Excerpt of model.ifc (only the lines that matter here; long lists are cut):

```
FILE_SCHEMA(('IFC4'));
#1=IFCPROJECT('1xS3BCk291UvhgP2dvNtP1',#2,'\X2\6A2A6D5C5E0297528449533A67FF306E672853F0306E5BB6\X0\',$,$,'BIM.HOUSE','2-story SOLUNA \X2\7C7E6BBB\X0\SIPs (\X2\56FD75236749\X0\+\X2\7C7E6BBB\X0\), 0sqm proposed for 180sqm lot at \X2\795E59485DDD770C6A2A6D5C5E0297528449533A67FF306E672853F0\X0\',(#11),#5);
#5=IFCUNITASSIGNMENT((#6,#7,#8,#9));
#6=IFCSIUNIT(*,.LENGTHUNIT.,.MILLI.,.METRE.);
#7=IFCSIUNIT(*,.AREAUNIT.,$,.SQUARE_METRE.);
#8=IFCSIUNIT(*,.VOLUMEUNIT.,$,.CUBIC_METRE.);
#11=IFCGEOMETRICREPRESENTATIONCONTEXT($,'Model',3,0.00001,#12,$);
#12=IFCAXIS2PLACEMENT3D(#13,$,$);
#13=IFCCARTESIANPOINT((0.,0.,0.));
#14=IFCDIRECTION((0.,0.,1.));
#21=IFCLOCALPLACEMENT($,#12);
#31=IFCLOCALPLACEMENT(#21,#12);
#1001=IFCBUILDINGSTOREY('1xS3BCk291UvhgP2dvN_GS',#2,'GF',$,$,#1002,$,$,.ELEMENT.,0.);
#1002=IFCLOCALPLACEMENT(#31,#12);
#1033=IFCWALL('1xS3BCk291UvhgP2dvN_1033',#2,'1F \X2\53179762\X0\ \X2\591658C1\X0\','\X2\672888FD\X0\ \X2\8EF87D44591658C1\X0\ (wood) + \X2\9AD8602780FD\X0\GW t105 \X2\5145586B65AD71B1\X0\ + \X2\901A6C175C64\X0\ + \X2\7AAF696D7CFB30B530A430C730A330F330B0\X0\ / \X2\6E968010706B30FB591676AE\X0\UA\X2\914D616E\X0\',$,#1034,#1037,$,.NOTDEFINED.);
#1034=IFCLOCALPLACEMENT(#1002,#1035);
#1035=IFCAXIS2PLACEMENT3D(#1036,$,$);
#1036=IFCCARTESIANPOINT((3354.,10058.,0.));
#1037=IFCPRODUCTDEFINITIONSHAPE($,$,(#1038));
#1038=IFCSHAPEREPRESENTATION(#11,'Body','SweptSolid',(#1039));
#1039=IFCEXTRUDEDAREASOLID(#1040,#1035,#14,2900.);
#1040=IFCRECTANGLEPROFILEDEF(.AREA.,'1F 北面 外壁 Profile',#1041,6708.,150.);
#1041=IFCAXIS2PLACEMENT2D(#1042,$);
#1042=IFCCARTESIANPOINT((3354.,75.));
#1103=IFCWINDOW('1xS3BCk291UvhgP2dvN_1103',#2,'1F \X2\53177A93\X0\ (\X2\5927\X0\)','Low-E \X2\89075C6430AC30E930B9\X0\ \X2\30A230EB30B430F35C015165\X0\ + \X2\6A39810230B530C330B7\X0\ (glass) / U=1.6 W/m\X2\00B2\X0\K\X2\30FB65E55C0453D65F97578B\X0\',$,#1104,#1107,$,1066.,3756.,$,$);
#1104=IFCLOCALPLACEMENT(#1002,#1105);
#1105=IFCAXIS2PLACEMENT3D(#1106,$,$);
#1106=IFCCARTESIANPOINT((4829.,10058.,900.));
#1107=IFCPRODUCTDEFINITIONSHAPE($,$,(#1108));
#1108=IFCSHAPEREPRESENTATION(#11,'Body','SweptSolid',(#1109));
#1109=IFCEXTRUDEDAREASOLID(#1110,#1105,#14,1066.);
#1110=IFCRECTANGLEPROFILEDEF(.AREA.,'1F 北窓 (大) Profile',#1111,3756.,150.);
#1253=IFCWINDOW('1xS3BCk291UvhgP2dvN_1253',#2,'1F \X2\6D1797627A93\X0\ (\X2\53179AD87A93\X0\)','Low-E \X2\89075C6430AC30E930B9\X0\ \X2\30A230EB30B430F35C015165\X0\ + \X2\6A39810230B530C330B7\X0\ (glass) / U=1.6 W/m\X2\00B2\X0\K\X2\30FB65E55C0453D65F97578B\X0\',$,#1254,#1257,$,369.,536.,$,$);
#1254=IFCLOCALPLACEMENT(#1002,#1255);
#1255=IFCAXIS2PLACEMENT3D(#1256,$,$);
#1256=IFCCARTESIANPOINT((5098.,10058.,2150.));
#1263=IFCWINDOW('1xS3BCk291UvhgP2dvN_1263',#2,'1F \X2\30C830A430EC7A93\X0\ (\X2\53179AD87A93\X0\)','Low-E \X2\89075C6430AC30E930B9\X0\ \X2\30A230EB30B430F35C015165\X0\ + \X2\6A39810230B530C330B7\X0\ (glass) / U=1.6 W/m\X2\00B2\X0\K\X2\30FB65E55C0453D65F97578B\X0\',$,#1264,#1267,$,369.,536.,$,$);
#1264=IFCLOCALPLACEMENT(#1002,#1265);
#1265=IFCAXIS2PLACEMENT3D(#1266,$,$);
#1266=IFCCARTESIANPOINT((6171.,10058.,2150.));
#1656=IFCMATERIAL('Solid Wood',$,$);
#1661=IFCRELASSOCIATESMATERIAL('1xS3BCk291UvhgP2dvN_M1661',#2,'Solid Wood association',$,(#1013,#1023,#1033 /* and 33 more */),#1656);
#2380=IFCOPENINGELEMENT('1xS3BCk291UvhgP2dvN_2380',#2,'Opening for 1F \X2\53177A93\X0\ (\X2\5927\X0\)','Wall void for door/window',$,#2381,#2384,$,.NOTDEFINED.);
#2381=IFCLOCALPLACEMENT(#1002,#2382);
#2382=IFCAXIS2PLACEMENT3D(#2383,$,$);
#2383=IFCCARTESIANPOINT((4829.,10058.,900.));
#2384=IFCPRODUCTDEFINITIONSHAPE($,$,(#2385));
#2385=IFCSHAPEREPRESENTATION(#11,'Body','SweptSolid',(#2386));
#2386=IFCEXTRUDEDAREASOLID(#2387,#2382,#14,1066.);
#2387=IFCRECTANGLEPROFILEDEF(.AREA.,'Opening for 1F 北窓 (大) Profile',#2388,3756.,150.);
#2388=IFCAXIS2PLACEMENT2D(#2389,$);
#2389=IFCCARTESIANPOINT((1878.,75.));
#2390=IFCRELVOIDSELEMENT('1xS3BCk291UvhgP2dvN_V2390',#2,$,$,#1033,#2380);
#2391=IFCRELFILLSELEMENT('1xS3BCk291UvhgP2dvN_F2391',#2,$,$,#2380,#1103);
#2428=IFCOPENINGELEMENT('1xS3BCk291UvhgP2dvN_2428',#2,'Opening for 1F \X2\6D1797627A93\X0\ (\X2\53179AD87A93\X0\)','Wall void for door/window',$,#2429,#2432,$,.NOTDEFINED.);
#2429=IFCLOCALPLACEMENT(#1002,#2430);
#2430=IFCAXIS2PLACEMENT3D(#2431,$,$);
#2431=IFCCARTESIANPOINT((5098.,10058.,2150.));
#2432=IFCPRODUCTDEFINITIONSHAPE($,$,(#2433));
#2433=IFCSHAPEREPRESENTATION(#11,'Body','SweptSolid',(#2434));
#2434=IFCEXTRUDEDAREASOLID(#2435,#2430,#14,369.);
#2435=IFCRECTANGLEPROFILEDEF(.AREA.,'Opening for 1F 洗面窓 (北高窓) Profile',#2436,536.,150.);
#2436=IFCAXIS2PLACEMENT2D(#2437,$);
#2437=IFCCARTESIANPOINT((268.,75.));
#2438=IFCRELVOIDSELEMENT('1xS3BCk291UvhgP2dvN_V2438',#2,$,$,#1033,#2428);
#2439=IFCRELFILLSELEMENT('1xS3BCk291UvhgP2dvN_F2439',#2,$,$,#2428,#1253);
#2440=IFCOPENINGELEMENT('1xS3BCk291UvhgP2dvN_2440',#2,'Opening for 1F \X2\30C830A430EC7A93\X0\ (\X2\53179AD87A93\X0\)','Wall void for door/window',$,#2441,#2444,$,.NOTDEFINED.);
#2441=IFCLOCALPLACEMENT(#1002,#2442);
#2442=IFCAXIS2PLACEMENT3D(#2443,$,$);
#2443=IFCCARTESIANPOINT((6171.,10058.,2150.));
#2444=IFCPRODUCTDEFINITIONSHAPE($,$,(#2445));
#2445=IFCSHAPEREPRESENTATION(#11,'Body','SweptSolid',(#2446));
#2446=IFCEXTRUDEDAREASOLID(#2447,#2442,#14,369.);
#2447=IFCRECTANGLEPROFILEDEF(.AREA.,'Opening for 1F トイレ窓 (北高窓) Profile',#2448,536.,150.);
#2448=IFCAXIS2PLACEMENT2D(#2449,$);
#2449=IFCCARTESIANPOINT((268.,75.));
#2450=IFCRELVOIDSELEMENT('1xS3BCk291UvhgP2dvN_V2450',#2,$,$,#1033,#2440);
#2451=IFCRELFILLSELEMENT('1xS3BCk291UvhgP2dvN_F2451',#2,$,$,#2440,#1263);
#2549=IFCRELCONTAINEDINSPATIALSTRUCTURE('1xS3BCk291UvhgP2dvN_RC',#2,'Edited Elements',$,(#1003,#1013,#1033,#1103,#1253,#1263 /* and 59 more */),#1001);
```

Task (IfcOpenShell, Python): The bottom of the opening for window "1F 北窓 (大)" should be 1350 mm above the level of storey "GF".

```python
import numpy as np
import ifcopenshell
import ifcopenshell.api.geometry
import ifcopenshell.geom
import ifcopenshell.util.element
import ifcopenshell.util.placement
import ifcopenshell.util.shape
import ifcopenshell.util.unit

model = ifcopenshell.open("model.ifc")
unit_scale = ifcopenshell.util.unit.calculate_unit_scale(model)

window = model.by_id(1103)
opening = window.FillsVoids[0].RelatingOpeningElement
storey = ifcopenshell.util.element.get_container(window, ifc_class="IfcBuildingStorey")
level = ifcopenshell.util.placement.get_local_placement(storey.ObjectPlacement)[2, 3]

# The opening's origin need not be at the sill, so measure its lowest point.
shape = ifcopenshell.geom.create_shape(ifcopenshell.geom.settings(), opening)
bottom = ifcopenshell.util.shape.get_shape_bottom_elevation(shape, shape.geometry) / unit_scale
dz = level + 1.35 / unit_scale - bottom

shift = np.array([0.0, 0.0, dz])
# The window is not placed relative to its opening, so move both.
for product in (opening, window):
    matrix = ifcopenshell.util.placement.get_local_placement(product.ObjectPlacement)
    matrix[:3, 3] += shift
    ifcopenshell.api.geometry.edit_object_placement(model, product=product, matrix=matrix, is_si=False)

print(f"moved by {dz * unit_scale:+.3f} m")

model.write("model_rev.ifc")
```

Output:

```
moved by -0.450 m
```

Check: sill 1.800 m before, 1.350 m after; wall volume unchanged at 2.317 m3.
